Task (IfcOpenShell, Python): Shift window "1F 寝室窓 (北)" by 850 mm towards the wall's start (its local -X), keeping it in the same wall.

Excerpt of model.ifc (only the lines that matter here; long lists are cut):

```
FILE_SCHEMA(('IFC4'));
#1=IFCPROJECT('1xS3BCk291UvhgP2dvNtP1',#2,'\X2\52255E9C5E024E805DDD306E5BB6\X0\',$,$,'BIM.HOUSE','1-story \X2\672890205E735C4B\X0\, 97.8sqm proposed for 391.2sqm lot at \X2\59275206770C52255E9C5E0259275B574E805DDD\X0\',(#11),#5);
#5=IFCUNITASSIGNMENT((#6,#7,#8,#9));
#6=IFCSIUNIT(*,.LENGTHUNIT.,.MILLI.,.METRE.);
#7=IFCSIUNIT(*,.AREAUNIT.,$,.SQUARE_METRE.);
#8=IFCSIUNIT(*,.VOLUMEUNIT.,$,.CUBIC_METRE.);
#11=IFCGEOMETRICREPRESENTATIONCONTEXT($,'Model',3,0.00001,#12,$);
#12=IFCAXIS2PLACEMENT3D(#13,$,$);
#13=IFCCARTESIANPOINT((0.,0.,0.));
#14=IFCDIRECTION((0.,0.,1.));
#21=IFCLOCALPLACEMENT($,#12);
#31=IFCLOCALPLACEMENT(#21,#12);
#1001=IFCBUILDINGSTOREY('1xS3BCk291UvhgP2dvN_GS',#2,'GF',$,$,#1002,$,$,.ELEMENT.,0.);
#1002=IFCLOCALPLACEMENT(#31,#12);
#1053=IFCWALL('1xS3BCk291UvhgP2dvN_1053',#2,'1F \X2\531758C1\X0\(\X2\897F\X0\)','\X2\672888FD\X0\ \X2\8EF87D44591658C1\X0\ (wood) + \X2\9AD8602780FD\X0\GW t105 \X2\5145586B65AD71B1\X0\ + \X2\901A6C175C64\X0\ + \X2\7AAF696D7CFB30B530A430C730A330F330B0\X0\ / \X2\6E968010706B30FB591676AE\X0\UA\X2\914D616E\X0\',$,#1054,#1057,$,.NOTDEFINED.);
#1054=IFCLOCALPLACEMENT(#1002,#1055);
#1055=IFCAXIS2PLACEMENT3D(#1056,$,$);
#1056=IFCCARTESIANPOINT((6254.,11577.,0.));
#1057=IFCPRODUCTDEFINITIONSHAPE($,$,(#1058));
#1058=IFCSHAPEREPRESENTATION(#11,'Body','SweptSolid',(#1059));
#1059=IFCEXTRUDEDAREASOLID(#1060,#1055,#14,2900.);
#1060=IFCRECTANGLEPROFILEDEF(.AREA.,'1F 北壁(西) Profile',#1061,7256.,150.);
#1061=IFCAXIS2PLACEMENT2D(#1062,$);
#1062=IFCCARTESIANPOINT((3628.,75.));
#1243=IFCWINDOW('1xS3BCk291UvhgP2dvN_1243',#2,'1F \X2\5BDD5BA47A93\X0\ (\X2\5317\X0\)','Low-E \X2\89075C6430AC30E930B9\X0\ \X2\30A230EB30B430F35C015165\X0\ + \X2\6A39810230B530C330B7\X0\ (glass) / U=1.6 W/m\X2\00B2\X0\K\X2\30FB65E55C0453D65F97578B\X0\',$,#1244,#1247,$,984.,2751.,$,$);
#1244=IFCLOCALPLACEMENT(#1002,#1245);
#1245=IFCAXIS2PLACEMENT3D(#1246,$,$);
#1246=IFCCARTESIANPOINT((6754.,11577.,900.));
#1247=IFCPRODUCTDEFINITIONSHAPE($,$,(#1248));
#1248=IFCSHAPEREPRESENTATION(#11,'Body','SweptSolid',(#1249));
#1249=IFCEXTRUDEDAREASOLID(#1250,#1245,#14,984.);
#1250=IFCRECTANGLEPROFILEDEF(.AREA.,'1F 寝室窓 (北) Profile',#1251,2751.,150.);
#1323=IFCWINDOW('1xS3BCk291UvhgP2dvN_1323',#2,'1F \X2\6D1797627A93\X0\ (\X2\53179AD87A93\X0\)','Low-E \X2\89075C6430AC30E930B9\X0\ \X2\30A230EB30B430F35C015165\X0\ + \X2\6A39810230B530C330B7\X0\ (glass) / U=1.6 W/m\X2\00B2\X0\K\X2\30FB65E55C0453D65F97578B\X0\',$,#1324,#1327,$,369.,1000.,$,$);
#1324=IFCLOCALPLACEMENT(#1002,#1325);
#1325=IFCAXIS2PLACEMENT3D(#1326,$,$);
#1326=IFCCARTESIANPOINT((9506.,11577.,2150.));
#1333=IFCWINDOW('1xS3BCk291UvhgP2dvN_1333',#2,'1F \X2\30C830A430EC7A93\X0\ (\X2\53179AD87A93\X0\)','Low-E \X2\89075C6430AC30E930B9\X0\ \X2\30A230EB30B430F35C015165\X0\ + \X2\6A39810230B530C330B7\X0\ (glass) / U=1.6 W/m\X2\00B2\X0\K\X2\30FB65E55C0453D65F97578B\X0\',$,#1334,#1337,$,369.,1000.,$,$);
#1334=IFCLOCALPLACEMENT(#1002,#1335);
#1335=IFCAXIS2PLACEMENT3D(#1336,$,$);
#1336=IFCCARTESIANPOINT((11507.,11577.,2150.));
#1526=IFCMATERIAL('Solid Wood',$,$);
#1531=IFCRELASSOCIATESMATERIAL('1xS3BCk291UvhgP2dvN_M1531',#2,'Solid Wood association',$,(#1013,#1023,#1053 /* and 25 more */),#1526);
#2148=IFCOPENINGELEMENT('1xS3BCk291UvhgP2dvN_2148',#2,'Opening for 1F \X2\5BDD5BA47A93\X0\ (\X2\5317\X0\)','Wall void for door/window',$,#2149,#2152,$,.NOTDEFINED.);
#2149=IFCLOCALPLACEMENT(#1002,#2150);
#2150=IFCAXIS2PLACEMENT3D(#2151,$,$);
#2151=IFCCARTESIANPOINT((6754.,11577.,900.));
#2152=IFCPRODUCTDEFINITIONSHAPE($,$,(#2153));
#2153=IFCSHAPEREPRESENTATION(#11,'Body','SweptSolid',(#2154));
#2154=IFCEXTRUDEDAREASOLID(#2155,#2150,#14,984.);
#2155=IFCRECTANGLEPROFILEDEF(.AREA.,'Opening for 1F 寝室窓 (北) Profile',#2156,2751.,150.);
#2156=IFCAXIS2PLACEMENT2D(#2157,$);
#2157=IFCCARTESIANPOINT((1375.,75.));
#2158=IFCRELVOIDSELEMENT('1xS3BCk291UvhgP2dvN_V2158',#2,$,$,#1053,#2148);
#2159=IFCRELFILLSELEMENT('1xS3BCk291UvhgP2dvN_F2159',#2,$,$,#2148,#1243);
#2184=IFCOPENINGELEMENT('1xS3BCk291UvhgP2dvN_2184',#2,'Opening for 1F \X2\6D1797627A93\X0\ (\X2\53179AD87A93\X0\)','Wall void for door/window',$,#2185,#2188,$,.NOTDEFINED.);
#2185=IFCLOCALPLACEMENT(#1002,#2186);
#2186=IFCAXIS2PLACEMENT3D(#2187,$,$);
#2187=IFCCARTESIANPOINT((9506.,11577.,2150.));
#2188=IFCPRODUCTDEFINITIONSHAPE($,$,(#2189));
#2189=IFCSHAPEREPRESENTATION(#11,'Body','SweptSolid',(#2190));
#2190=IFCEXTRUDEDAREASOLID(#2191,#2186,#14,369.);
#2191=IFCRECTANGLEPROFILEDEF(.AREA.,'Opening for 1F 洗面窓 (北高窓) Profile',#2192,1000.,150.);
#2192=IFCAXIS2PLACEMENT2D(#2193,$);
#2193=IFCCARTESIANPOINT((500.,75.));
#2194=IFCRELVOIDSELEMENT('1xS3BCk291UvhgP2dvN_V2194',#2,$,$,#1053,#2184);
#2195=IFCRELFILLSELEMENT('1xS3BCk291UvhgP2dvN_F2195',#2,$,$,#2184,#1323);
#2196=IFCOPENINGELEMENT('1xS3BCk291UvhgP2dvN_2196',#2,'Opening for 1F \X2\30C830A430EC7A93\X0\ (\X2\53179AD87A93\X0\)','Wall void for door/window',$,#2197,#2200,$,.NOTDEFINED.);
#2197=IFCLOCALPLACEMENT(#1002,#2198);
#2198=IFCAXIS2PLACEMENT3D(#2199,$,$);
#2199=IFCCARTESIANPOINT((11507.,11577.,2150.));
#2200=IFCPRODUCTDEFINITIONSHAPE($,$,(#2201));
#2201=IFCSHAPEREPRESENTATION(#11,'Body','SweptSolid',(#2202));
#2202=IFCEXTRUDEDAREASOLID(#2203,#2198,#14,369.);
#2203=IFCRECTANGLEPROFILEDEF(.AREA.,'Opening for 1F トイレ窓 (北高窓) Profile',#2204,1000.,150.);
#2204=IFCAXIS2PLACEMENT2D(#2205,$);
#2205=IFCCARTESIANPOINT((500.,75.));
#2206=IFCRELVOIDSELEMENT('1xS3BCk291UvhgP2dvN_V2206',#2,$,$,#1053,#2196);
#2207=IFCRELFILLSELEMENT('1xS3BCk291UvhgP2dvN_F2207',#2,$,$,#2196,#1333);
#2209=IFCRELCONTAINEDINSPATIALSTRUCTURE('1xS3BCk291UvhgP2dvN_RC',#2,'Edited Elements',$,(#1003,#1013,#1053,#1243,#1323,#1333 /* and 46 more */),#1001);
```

```python
import ifcopenshell
import ifcopenshell.api.geometry
import ifcopenshell.util.placement
import ifcopenshell.util.unit

model = ifcopenshell.open("model.ifc")
unit_scale = ifcopenshell.util.unit.calculate_unit_scale(model)

window = model.by_id(1243)
opening = window.FillsVoids[0].RelatingOpeningElement
wall = opening.VoidsElements[0].RelatingBuildingElement

wall_matrix = ifcopenshell.util.placement.get_local_placement(wall.ObjectPlacement)
shift = wall_matrix[:3, 0] * -0.85 / unit_scale
before = ifcopenshell.util.placement.get_local_placement(window.ObjectPlacement)[:3, 3].copy()

# The window is not placed relative to its opening, so move both.
for product in (opening, window):
    matrix = ifcopenshell.util.placement.get_local_placement(product.ObjectPlacement)
    matrix[:3, 3] += shift
    ifcopenshell.api.geometry.edit_object_placement(model, product=product, matrix=matrix, is_si=False)

after = ifcopenshell.util.placement.get_local_placement(window.ObjectPlacement)[:3, 3]
print("window moved by", (after - before).round(3) + 0.0)

model.write("model_edited.ifc")
```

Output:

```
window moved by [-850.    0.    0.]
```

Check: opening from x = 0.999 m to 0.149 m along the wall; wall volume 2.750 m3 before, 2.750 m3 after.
